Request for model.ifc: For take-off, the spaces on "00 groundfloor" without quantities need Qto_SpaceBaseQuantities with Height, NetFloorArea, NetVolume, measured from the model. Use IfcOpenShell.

First a look at what the model holds.

```python
import ifcopenshell
import ifcopenshell.util.element
import ifcopenshell.util.unit

model = ifcopenshell.open("model.ifc")
print(model.schema)
for unit_type in ("LENGTHUNIT", "AREAUNIT", "VOLUMEUNIT"):
    print(unit_type, ifcopenshell.util.unit.calculate_unit_scale(model, unit_type))
storey = next(s for s in model.by_type("IfcBuildingStorey") if s.Name == "00 groundfloor")
spaces = [e for e in ifcopenshell.util.element.get_decomposition(storey) if e.is_a("IfcSpace")]
for e in sorted(spaces, key=lambda e: e.id()):
    print(e.id(), e.is_a(), e.Name, list(ifcopenshell.util.element.get_psets(e, qtos_only=True)), sep=" | ")
```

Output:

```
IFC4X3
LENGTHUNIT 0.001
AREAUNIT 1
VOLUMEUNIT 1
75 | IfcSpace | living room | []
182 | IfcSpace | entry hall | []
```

```python
import ifcopenshell
import ifcopenshell.api.pset
import ifcopenshell.geom
import ifcopenshell.util.element
import ifcopenshell.util.shape
import ifcopenshell.util.unit

model = ifcopenshell.open("model.ifc")
unit_scale = ifcopenshell.util.unit.calculate_unit_scale(model)
area_scale = ifcopenshell.util.unit.calculate_unit_scale(model, "AREAUNIT")
volume_scale = ifcopenshell.util.unit.calculate_unit_scale(model, "VOLUMEUNIT")
settings = ifcopenshell.geom.settings()

storey = next(s for s in model.by_type("IfcBuildingStorey") if s.Name == "00 groundfloor")
spaces = [e for e in ifcopenshell.util.element.get_decomposition(storey) if e.is_a("IfcSpace")]

for e in sorted(spaces, key=lambda e: e.id()):
    if ifcopenshell.util.element.get_psets(e, qtos_only=True, should_inherit=False):
        continue
    # Geometry comes back in metres, in the element's own axes.
    shape = ifcopenshell.geom.create_shape(settings, e)
    values = {
        "Height": ifcopenshell.util.shape.get_z(shape.geometry) / unit_scale,
        "NetFloorArea": ifcopenshell.util.shape.get_footprint_area(shape.geometry) / area_scale,
        "NetVolume": ifcopenshell.util.shape.get_volume(shape.geometry) / volume_scale,
    }
    qto = ifcopenshell.api.pset.add_qto(model, product=e, name="Qto_SpaceBaseQuantities")
    ifcopenshell.api.pset.edit_qto(model, qto=qto, properties=values)
    print(e.id(), {k: round(v, 3) for k, v in values.items()})

model.write("model_rev.ifc")
```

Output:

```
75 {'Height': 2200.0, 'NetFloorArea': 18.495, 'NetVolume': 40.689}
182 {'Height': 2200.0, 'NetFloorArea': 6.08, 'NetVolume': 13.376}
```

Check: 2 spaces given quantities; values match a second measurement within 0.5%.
